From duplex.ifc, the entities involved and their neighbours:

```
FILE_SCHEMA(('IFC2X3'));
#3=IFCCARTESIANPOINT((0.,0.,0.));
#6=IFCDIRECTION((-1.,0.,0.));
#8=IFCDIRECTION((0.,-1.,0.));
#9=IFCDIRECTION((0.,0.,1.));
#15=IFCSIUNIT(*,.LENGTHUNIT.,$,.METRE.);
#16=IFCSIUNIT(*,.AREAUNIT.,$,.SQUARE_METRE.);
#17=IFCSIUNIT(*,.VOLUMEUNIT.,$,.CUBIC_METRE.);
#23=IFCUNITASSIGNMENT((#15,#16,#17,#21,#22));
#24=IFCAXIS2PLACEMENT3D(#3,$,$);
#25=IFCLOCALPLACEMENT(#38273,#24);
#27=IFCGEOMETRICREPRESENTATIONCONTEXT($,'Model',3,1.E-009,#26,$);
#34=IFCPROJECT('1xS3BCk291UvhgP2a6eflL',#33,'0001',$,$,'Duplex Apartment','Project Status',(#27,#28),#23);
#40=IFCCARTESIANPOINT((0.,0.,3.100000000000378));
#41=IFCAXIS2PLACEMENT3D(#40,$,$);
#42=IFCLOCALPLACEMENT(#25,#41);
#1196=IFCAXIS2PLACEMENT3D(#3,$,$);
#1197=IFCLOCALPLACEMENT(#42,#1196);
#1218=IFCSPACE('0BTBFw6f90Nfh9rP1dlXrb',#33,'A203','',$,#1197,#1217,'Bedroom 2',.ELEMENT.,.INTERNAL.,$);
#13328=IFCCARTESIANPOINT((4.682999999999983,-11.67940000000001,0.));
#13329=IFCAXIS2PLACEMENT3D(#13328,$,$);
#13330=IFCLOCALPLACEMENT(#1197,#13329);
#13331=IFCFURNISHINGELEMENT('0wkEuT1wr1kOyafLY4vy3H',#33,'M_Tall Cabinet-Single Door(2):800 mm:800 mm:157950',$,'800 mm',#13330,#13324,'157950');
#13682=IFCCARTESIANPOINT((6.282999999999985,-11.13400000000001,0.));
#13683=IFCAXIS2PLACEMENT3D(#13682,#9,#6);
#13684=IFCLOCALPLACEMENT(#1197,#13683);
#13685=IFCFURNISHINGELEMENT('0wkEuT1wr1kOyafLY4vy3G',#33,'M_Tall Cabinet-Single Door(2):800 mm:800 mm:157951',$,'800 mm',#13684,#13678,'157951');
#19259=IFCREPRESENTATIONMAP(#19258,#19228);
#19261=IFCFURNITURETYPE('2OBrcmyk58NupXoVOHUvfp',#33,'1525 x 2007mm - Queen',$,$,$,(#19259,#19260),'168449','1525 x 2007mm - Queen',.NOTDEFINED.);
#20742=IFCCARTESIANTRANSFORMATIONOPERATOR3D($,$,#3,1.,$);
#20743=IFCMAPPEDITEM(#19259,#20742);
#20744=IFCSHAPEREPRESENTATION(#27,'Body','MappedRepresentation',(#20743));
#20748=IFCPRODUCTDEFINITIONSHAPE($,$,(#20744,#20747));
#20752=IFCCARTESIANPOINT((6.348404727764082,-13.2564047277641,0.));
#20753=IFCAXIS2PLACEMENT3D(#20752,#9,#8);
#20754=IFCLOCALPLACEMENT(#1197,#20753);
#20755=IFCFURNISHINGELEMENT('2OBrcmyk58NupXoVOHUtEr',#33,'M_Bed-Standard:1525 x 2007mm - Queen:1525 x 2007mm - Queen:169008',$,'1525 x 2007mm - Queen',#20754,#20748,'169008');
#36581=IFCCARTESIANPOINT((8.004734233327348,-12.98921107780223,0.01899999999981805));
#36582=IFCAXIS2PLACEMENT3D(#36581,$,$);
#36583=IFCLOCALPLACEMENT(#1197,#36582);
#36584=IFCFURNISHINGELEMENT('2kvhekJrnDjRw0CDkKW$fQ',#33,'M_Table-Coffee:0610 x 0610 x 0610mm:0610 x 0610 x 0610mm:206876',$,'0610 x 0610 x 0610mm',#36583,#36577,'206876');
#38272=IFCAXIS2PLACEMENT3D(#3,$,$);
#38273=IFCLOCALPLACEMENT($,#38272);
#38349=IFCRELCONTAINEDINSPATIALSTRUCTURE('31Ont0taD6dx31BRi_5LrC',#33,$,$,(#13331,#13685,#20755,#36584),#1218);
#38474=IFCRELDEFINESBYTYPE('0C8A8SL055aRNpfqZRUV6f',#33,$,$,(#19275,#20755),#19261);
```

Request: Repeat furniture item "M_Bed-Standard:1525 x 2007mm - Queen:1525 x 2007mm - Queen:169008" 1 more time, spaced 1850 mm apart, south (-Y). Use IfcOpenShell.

```python
import numpy as np
import ifcopenshell
import ifcopenshell.api.geometry
import ifcopenshell.api.root
import ifcopenshell.util.element
import ifcopenshell.util.placement
import ifcopenshell.util.unit

model = ifcopenshell.open("duplex.ifc")
unit_scale = ifcopenshell.util.unit.calculate_unit_scale(model)


def reuse_history(source, copy):
    """copy_class also copies each property set's owner history, people and application; keep the originals."""
    for rel in copy.IsDefinedBy:
        if rel.is_a("IfcRelDefinesByProperties") and (history := rel.RelatingPropertyDefinition.OwnerHistory):
            rel.RelatingPropertyDefinition.OwnerHistory = source.OwnerHistory
            ifcopenshell.util.element.remove_deep2(model, history)


source = model.by_guid("2OBrcmyk58NupXoVOHUtEr")
base = ifcopenshell.util.placement.get_local_placement(source.ObjectPlacement)
step = np.array([0.0, -1.0, 0.0]) * 1.85 / unit_scale

for i in range(1, 2):
    copy = ifcopenshell.api.root.copy_class(model, product=source)
    copy.Representation = ifcopenshell.util.element.copy_deep(
        model, source.Representation, exclude=["IfcGeometricRepresentationContext", "IfcRepresentationMap"]
    )
    copy.Name = "M_Bed-Standard:1525 x 2007mm - Queen:1525 x 2007mm - Queen"
    copy.Tag = None
    reuse_history(source, copy)
    matrix = base.copy()
    matrix[:3, 3] += i * step
    print("added at", matrix[:3, 3].round(3) + 0.0)
    ifcopenshell.api.geometry.edit_object_placement(model, product=copy, matrix=matrix, is_si=False)

model.write("duplex_updated.ifc")
```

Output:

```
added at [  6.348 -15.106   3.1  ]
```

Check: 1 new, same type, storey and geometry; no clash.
